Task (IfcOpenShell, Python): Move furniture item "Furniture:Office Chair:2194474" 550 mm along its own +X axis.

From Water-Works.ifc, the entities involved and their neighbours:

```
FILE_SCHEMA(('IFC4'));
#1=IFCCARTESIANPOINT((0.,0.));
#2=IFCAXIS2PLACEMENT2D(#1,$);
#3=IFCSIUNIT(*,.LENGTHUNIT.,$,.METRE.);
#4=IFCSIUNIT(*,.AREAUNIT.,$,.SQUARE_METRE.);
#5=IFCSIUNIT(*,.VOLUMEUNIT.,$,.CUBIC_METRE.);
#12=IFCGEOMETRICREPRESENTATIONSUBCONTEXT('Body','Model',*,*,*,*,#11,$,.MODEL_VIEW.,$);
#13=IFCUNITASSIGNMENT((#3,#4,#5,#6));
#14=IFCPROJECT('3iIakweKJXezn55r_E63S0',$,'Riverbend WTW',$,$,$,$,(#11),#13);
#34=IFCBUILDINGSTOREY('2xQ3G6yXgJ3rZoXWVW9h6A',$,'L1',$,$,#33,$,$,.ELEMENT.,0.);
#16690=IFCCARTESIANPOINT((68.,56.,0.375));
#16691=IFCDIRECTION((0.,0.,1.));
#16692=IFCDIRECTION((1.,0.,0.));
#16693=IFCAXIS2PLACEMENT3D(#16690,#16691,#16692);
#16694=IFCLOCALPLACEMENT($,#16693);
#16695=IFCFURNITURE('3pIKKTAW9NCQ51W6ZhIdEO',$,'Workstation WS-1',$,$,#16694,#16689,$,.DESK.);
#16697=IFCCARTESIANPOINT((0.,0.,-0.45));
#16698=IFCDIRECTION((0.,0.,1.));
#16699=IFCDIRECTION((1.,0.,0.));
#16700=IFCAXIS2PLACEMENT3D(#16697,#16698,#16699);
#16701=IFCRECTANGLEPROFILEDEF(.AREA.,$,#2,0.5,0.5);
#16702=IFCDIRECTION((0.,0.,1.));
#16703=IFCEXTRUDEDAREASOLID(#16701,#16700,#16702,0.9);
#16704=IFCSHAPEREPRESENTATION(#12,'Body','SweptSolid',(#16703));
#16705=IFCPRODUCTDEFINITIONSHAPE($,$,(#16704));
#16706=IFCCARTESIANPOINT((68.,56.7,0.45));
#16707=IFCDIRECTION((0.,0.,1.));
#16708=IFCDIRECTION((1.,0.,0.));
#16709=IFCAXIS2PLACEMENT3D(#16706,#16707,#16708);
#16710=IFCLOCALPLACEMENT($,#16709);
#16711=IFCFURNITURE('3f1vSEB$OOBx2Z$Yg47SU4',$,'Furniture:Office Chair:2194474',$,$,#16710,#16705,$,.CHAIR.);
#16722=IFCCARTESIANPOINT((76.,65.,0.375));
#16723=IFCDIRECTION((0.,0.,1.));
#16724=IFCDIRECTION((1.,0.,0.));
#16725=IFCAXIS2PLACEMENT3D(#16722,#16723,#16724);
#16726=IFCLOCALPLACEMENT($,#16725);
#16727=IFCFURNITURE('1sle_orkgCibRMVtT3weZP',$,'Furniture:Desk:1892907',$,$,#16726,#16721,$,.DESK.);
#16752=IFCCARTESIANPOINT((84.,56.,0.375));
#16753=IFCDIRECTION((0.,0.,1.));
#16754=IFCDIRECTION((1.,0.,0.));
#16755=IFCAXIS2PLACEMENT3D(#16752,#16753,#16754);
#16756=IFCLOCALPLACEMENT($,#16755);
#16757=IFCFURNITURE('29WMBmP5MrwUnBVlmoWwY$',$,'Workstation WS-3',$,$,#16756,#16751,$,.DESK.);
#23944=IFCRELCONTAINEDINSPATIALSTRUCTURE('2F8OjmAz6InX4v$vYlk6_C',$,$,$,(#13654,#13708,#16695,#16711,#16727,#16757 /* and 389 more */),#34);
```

```python
import ifcopenshell
import ifcopenshell.api.geometry
import ifcopenshell.util.placement

model = ifcopenshell.open("Water-Works.ifc")

item = model.by_guid("3f1vSEB$OOBx2Z$Yg47SU4")
matrix = ifcopenshell.util.placement.get_local_placement(item.ObjectPlacement)
matrix[:3, 3] += matrix[:3, 0] * 0.55
ifcopenshell.api.geometry.edit_object_placement(model, product=item, matrix=matrix, is_si=False)

print(ifcopenshell.util.placement.get_local_placement(item.ObjectPlacement).round(3) + 0.0)

model.write("Water-Works_updated.ifc")
```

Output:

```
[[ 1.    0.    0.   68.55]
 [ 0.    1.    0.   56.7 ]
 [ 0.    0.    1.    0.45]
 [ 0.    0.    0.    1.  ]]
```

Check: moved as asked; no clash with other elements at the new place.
